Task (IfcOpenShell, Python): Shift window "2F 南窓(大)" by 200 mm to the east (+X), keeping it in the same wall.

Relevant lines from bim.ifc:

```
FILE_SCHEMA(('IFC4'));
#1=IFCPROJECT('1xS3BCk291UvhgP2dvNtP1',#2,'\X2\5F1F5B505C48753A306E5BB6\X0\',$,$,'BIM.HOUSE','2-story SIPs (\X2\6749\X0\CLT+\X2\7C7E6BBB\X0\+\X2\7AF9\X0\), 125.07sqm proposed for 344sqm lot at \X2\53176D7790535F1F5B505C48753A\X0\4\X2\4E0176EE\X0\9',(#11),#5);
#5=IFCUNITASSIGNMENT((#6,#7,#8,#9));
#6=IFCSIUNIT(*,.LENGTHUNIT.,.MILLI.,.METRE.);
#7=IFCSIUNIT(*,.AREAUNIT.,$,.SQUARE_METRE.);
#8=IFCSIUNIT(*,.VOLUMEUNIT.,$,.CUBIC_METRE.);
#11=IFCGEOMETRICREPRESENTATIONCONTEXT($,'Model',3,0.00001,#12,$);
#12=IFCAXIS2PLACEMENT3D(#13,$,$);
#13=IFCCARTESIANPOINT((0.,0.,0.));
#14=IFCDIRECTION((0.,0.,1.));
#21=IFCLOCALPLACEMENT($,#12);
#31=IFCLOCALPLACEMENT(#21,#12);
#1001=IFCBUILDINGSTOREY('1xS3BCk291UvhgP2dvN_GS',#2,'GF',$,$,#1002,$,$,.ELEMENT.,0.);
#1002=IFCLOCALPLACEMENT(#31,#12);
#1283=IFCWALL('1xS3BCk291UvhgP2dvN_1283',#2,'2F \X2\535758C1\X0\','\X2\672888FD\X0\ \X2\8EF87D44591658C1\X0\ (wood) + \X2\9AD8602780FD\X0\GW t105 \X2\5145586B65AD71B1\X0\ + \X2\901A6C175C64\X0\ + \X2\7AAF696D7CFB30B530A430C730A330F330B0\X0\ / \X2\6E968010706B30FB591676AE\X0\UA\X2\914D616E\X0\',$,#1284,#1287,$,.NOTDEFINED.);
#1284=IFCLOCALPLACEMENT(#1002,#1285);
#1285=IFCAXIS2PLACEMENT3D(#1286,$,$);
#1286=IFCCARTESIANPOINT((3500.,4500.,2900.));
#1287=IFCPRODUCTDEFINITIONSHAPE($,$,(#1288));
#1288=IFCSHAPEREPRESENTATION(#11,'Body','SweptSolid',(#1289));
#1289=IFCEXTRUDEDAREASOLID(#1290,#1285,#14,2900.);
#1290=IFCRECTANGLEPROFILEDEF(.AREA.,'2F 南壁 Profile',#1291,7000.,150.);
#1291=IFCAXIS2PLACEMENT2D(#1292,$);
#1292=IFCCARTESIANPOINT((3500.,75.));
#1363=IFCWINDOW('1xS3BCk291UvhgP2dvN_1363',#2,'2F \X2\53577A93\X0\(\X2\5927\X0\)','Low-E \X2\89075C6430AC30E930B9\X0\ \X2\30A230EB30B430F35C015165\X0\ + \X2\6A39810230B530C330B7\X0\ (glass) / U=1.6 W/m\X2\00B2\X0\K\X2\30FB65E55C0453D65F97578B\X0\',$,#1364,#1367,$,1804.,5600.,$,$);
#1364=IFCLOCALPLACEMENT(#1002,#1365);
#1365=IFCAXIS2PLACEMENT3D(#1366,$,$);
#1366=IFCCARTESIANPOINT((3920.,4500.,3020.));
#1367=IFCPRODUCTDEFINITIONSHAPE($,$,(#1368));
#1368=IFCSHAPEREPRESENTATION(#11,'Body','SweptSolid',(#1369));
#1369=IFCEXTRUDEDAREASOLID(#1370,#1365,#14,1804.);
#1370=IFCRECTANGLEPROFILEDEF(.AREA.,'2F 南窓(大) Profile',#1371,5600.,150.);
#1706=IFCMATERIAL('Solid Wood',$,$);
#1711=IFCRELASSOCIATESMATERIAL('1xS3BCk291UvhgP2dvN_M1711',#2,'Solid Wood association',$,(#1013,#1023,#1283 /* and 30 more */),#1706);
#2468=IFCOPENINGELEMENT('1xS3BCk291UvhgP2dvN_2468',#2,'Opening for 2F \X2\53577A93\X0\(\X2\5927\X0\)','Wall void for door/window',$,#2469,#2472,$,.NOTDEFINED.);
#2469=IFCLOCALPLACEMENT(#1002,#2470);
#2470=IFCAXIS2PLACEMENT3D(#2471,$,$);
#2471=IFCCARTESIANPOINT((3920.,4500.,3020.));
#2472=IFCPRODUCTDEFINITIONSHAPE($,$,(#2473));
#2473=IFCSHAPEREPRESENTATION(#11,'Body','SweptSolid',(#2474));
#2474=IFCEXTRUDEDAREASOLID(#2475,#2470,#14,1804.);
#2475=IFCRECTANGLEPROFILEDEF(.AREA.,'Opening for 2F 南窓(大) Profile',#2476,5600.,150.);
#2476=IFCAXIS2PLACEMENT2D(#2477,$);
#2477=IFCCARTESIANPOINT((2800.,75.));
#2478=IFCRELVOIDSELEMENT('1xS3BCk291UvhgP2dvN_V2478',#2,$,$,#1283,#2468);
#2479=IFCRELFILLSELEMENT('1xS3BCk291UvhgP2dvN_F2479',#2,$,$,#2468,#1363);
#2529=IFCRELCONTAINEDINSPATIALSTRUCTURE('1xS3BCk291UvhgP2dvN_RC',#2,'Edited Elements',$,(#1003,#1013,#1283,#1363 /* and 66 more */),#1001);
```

```python
import ifcopenshell
import ifcopenshell.api.geometry
import ifcopenshell.util.placement

model = ifcopenshell.open("bim.ifc")

window = model.by_guid("1xS3BCk291UvhgP2dvN_1363")
opening = window.FillsVoids[0].RelatingOpeningElement
wall = opening.VoidsElements[0].RelatingBuildingElement

wall_matrix = ifcopenshell.util.placement.get_local_placement(wall.ObjectPlacement)
shift = wall_matrix[:3, 0] * 200.0
before = ifcopenshell.util.placement.get_local_placement(window.ObjectPlacement)[:3, 3].copy()

# The window is not placed relative to its opening, so move both.
for product in (opening, window):
    matrix = ifcopenshell.util.placement.get_local_placement(product.ObjectPlacement)
    matrix[:3, 3] += shift
    ifcopenshell.api.geometry.edit_object_placement(model, product=product, matrix=matrix, is_si=False)

after = ifcopenshell.util.placement.get_local_placement(window.ObjectPlacement)[:3, 3]
print("window moved by", (after - before).round(3) + 0.0)

model.write("bim_edited.ifc")
```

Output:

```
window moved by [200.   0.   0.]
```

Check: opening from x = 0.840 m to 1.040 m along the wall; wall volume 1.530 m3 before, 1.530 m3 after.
